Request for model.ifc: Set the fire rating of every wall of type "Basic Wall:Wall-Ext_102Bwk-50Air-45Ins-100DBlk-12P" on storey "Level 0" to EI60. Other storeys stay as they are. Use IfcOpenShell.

First a look at what the model holds.

```python
import ifcopenshell
import ifcopenshell.util.element

model = ifcopenshell.open("model.ifc")
print(model.schema)
storey = next(s for s in model.by_type("IfcBuildingStorey") if s.Name == "Level 0")
walls = [e for e in ifcopenshell.util.element.get_decomposition(storey) if e.is_a("IfcWall")]
seen = {}
for e in walls:
    element_type = ifcopenshell.util.element.get_type(e)
    key = (element_type.Name if element_type != e and element_type else None, ifcopenshell.util.element.get_pset(e, "Pset_WallCommon", "FireRating"))
    seen[key] = seen.get(key, 0) + 1
for (name, value), count in sorted(seen.items(), key=str):
    print(count, "x", name, "|", value)
```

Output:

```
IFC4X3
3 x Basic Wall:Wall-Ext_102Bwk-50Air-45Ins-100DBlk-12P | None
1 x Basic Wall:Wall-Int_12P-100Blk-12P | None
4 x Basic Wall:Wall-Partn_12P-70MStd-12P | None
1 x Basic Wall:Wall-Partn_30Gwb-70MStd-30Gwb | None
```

```python
import ifcopenshell
import ifcopenshell.api.pset
import ifcopenshell.util.element

model = ifcopenshell.open("model.ifc")

storey = next(s for s in model.by_type("IfcBuildingStorey") if s.Name == "Level 0")
walls = [e for e in ifcopenshell.util.element.get_decomposition(storey) if e.is_a("IfcWall")]

count = 0
for e in walls:
    element_type = ifcopenshell.util.element.get_type(e)
    if element_type in (None, e) or element_type.Name != "Basic Wall:Wall-Ext_102Bwk-50Air-45Ins-100DBlk-12P":
        continue
    # add_pset returns the element's existing set when there is one.
    pset = ifcopenshell.api.pset.add_pset(model, product=e, name="Pset_WallCommon")
    ifcopenshell.api.pset.edit_pset(model, pset=pset, properties={"FireRating": "EI60"})
    count += 1

print(count, "walls updated")

model.write("model_v2.ifc")
```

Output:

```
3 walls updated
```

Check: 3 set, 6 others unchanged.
